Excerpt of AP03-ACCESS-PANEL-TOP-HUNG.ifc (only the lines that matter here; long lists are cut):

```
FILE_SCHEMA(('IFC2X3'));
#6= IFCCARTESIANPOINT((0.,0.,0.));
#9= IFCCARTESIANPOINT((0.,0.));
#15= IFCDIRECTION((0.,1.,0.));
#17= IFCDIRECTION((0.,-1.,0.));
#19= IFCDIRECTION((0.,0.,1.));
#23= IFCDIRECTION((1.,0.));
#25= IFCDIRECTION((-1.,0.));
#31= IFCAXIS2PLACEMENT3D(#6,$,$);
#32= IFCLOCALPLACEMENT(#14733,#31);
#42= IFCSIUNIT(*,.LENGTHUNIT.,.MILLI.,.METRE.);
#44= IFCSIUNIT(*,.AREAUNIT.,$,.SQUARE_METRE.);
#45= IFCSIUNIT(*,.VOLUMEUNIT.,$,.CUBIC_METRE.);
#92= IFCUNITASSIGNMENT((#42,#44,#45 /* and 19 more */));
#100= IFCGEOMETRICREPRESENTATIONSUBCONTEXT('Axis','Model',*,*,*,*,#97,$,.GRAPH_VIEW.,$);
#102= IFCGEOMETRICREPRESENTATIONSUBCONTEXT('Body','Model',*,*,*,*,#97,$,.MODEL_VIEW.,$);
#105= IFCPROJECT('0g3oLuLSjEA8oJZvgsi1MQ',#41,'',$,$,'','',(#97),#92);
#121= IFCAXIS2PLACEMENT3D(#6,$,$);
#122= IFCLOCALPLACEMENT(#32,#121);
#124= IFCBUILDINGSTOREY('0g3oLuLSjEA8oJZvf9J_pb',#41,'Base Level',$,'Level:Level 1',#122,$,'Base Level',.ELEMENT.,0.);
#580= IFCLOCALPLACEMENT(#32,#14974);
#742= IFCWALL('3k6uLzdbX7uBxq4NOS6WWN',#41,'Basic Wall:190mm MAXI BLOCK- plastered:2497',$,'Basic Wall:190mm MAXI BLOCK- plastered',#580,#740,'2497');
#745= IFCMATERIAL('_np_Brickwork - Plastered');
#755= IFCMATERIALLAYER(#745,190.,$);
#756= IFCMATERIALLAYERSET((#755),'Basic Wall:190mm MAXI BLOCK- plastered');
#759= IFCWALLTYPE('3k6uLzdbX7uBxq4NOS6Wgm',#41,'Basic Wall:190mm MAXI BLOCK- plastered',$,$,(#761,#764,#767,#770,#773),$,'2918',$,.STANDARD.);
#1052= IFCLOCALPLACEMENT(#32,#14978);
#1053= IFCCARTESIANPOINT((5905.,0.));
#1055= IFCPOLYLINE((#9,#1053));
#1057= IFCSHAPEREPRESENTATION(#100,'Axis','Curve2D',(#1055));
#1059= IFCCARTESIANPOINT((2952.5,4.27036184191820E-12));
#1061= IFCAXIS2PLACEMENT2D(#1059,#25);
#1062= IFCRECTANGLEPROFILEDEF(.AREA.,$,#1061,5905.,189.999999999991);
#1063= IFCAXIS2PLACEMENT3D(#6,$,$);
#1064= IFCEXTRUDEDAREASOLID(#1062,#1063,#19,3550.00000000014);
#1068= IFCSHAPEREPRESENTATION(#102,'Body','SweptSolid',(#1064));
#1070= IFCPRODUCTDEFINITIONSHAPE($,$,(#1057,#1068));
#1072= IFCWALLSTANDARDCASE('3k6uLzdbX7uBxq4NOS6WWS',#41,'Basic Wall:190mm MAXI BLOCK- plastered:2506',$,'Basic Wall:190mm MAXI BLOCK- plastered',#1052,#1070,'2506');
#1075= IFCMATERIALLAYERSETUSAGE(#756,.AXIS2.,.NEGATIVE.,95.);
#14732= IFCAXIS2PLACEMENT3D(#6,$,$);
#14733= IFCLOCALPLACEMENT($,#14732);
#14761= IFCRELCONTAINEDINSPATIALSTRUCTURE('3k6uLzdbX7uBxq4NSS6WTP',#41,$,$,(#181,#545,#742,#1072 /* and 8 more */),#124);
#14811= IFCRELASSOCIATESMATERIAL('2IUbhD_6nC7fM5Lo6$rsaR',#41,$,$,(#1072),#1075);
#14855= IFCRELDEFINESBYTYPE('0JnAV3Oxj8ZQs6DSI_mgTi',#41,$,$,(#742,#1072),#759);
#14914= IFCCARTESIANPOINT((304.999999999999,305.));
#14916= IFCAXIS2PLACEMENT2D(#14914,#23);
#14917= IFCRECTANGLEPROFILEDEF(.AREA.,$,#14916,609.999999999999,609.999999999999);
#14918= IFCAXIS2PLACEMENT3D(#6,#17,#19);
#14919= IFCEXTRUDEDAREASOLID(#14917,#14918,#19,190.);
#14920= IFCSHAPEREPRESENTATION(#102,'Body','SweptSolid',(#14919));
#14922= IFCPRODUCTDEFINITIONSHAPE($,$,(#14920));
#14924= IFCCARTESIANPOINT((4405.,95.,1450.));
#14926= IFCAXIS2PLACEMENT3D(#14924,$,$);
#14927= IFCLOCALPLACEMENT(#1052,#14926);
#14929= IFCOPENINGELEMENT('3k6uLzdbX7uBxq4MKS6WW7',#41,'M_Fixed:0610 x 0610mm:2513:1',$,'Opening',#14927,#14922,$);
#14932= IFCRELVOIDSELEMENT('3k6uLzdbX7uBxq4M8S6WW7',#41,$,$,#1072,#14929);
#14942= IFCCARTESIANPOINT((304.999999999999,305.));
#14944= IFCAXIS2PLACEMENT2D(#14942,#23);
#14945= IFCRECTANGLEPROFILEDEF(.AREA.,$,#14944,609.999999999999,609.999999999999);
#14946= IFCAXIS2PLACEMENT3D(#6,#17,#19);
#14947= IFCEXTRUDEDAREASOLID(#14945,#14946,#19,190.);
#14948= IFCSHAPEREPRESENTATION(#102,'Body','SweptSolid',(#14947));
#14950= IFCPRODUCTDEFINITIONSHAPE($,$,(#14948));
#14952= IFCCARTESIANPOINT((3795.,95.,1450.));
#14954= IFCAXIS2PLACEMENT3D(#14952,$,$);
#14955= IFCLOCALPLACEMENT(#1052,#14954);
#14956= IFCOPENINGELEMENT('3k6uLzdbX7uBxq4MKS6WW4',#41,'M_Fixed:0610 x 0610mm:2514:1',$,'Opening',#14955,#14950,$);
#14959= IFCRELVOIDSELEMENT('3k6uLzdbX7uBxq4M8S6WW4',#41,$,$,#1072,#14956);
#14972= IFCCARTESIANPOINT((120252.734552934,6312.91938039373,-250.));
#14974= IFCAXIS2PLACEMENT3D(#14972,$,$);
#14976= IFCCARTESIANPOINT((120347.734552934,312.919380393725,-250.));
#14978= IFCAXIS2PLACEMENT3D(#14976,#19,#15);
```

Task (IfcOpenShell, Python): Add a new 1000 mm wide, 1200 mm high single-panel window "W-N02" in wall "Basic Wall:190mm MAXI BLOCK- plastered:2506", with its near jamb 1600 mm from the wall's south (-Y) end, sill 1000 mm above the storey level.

```python
import numpy as np
import ifcopenshell
import ifcopenshell.api.feature
import ifcopenshell.api.geometry
import ifcopenshell.api.root
import ifcopenshell.api.spatial
import ifcopenshell.api.type
import ifcopenshell.geom
import ifcopenshell.util.element
import ifcopenshell.util.placement
import ifcopenshell.util.representation
import ifcopenshell.util.shape
import ifcopenshell.util.unit

model = ifcopenshell.open("AP03-ACCESS-PANEL-TOP-HUNG.ifc")
unit_scale = ifcopenshell.util.unit.calculate_unit_scale(model)
settings = ifcopenshell.geom.settings()


def volume(element):
    """Net volume in cubic metres, openings subtracted."""
    shape = ifcopenshell.geom.create_shape(settings, element)
    return ifcopenshell.util.shape.get_volume(shape.geometry)


wall = model.by_id(1072)
storey = ifcopenshell.util.element.get_container(wall, ifc_class="IfcBuildingStorey")
context = ifcopenshell.util.representation.get_context(model, "Model", "Body", "MODEL_VIEW")
before = volume(wall)

width, height, from_end, sill = 1, 1.2, 1.6, 1  # metres

# The wall runs along its own X axis, and the end named is its -X end.
wall_shape = ifcopenshell.geom.create_shape(settings, wall)
x, y, z = ifcopenshell.util.shape.get_vertices(wall_shape.geometry).T
start = x.min() + from_end
face, thickness = float(y.min()), float(y.max() - y.min())
wall_matrix = ifcopenshell.util.placement.get_local_placement(wall.ObjectPlacement)
level = ifcopenshell.util.placement.get_local_placement(storey.ObjectPlacement)[2, 3]


def in_wall(x, y):
    """Placement at x, y metres in the wall's axes, at sill height."""
    matrix = wall_matrix.copy()
    matrix[:, 3] = wall_matrix @ np.array([x / unit_scale, y / unit_scale, 0.0, 1.0])
    matrix[2, 3] = level + sill / unit_scale
    return matrix


# Opening: a box that overshoots both wall faces by 50 mm.
opening = ifcopenshell.api.root.create_entity(model, ifc_class="IfcOpeningElement")
box = ifcopenshell.api.geometry.add_wall_representation(
    model, context=context, length=width, height=height, thickness=thickness + 0.1
)
ifcopenshell.api.geometry.assign_representation(model, product=opening, representation=box)
ifcopenshell.api.geometry.edit_object_placement(model, product=opening, matrix=in_wall(start, face - 0.05), is_si=False)
ifcopenshell.api.feature.add_feature(model, feature=opening, element=wall)

window = ifcopenshell.api.root.create_entity(model, ifc_class="IfcWindow", name="W-N02")
window.OverallWidth, window.OverallHeight = width / unit_scale, height / unit_scale
body = ifcopenshell.api.geometry.add_window_representation(
    model,
    context=context,
    overall_width=window.OverallWidth,
    overall_height=window.OverallHeight,
    partition_type="SINGLE_PANEL",
)
ifcopenshell.api.geometry.assign_representation(model, product=window, representation=body)
ifcopenshell.api.spatial.assign_container(model, products=[window], relating_structure=storey)
fills = ifcopenshell.api.feature.add_filling(model, opening=opening, element=window)
fills.OwnerHistory = window.OwnerHistory  # required in IFC2X3

# IFC2X3 keeps the operation on the window style.
style = ifcopenshell.api.root.create_entity(model, ifc_class="IfcWindowStyle", name="W-N02")
style.OperationType, style.ConstructionType = "SINGLE_PANEL", "NOTDEFINED"
style.ParameterTakesPrecedence = style.Sizeable = False
ifcopenshell.api.type.assign_type(model, related_objects=[window], relating_type=style)

# Centre the window in the wall's thickness.
ifcopenshell.api.geometry.edit_object_placement(model, product=window, matrix=in_wall(start, face), is_si=False)
window_shape = ifcopenshell.geom.create_shape(settings, window)
depth = ifcopenshell.util.shape.get_vertices(window_shape.geometry)[:, 1]
offset = face + thickness / 2 - (depth.min() + depth.max()) / 2
ifcopenshell.api.geometry.edit_object_placement(model, product=window, matrix=in_wall(start, offset), is_si=False)

after = volume(wall)

print(f"wall volume {before:.3f} -> {after:.3f} m3")

model.write("AP03-ACCESS-PANEL-TOP-HUNG_edited.ifc")
```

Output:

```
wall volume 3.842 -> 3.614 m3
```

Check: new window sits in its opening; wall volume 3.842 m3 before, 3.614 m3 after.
